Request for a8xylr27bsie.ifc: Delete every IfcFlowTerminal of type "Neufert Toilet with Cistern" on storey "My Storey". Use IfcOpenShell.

First a look at what the model holds.

```python
import ifcopenshell
import ifcopenshell.util.element

model = ifcopenshell.open("a8xylr27bsie.ifc")
print(model.schema)
storey = next(s for s in model.by_type("IfcBuildingStorey") if s.Name == "My Storey")
terminals = [e for e in ifcopenshell.util.element.get_decomposition(storey) if e.is_a("IfcFlowTerminal")]
seen = {}
for e in terminals:
    element_type = ifcopenshell.util.element.get_type(e)
    name = element_type.Name if element_type not in (None, e) else None
    seen[name] = seen.get(name, 0) + 1
for name, count in sorted(seen.items(), key=str):
    print(count, "x", name)
```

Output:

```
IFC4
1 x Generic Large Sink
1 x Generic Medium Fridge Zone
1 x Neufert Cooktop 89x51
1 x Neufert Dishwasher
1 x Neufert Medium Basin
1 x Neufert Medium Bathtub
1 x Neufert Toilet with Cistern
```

```python
import ifcopenshell
import ifcopenshell.api.root
import ifcopenshell.util.element

model = ifcopenshell.open("a8xylr27bsie.ifc")

storey = next(s for s in model.by_type("IfcBuildingStorey") if s.Name == "My Storey")
terminals = [e for e in ifcopenshell.util.element.get_decomposition(storey) if e.is_a("IfcFlowTerminal")]
targets = [e for e in terminals if (t := ifcopenshell.util.element.get_type(e)) not in (None, e) and t.Name == "Neufert Toilet with Cistern"]

for e in targets:
    ifcopenshell.api.root.remove_product(model, product=e)
print(len(targets), "removed")

model.write("a8xylr27bsie-out.ifc")
```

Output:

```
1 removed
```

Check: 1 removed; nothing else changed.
